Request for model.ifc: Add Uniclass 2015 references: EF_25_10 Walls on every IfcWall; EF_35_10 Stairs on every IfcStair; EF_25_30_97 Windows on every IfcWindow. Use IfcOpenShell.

First a look at what the model holds.

```python
import ifcopenshell

model = ifcopenshell.open("model.ifc")
print(model.schema)
print("classifications:", [c.Name for c in model.by_type("IfcClassification")])
for ifc_class in ("IfcDoor", "IfcRoof", "IfcStair", "IfcWall", "IfcWindow"):
    print(ifc_class, len(model.by_type(ifc_class)))
```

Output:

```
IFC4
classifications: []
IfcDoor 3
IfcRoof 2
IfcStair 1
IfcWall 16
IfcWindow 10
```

```python
import ifcopenshell
import ifcopenshell.api.classification

model = ifcopenshell.open("model.ifc")

system = ifcopenshell.api.classification.add_classification(model, classification="Uniclass 2015")

codes = {
    "IfcWall": ("EF_25_10", "Walls"),
    "IfcStair": ("EF_35_10", "Stairs"),
    "IfcWindow": ("EF_25_30_97", "Windows"),
}
for ifc_class, (code, name) in codes.items():
    products = model.by_type(ifc_class)
    ifcopenshell.api.classification.add_reference(
        model, products=products, classification=system, identification=code, name=name
    )
    print(code, len(products))

model.write("model_edited.ifc")
```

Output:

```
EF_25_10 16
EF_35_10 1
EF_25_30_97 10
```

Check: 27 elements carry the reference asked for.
